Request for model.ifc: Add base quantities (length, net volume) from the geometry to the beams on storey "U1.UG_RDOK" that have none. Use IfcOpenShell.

First a look at what the model holds.

```python
import ifcopenshell
import ifcopenshell.util.element
import ifcopenshell.util.unit

model = ifcopenshell.open("model.ifc")
print(model.schema)
for unit_type in ("LENGTHUNIT", "AREAUNIT", "VOLUMEUNIT"):
    print(unit_type, ifcopenshell.util.unit.calculate_unit_scale(model, unit_type))
storey = next(s for s in model.by_type("IfcBuildingStorey") if s.Name == "U1.UG_RDOK")
beams = [e for e in ifcopenshell.util.element.get_decomposition(storey) if e.is_a("IfcBeam")]
for e in sorted(beams, key=lambda e: e.id()):
    print(e.id(), e.is_a(), e.Name, list(ifcopenshell.util.element.get_psets(e, qtos_only=True)), sep=" | ")
```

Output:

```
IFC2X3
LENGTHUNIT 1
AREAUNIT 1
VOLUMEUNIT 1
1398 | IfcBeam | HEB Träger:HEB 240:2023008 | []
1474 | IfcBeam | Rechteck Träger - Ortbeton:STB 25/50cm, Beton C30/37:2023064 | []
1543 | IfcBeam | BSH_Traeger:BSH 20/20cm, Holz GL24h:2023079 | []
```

```python
import ifcopenshell
import ifcopenshell.api.pset
import ifcopenshell.geom
import ifcopenshell.util.element
import ifcopenshell.util.shape
import ifcopenshell.util.unit

model = ifcopenshell.open("model.ifc")
unit_scale = ifcopenshell.util.unit.calculate_unit_scale(model)
volume_scale = ifcopenshell.util.unit.calculate_unit_scale(model, "VOLUMEUNIT")
settings = ifcopenshell.geom.settings()

storey = next(s for s in model.by_type("IfcBuildingStorey") if s.Name == "U1.UG_RDOK")
beams = [e for e in ifcopenshell.util.element.get_decomposition(storey) if e.is_a("IfcBeam")]

for e in sorted(beams, key=lambda e: e.id()):
    if ifcopenshell.util.element.get_psets(e, qtos_only=True, should_inherit=False):
        continue
    # Geometry comes back in metres, in the element's own axes.
    shape = ifcopenshell.geom.create_shape(settings, e)
    values = {
        "Length": ifcopenshell.util.shape.get_max_xyz(shape.geometry) / unit_scale,
        "NetVolume": ifcopenshell.util.shape.get_volume(shape.geometry) / volume_scale,
    }
    qto = ifcopenshell.api.pset.add_qto(model, product=e, name="BaseQuantities")
    ifcopenshell.api.pset.edit_qto(model, qto=qto, properties=values)
    print(e.id(), {k: round(v, 3) for k, v in values.items()})

model.write("model-out.ifc")
```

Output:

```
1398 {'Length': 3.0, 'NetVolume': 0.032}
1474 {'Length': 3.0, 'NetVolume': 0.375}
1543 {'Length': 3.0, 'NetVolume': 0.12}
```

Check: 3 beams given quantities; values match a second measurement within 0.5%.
